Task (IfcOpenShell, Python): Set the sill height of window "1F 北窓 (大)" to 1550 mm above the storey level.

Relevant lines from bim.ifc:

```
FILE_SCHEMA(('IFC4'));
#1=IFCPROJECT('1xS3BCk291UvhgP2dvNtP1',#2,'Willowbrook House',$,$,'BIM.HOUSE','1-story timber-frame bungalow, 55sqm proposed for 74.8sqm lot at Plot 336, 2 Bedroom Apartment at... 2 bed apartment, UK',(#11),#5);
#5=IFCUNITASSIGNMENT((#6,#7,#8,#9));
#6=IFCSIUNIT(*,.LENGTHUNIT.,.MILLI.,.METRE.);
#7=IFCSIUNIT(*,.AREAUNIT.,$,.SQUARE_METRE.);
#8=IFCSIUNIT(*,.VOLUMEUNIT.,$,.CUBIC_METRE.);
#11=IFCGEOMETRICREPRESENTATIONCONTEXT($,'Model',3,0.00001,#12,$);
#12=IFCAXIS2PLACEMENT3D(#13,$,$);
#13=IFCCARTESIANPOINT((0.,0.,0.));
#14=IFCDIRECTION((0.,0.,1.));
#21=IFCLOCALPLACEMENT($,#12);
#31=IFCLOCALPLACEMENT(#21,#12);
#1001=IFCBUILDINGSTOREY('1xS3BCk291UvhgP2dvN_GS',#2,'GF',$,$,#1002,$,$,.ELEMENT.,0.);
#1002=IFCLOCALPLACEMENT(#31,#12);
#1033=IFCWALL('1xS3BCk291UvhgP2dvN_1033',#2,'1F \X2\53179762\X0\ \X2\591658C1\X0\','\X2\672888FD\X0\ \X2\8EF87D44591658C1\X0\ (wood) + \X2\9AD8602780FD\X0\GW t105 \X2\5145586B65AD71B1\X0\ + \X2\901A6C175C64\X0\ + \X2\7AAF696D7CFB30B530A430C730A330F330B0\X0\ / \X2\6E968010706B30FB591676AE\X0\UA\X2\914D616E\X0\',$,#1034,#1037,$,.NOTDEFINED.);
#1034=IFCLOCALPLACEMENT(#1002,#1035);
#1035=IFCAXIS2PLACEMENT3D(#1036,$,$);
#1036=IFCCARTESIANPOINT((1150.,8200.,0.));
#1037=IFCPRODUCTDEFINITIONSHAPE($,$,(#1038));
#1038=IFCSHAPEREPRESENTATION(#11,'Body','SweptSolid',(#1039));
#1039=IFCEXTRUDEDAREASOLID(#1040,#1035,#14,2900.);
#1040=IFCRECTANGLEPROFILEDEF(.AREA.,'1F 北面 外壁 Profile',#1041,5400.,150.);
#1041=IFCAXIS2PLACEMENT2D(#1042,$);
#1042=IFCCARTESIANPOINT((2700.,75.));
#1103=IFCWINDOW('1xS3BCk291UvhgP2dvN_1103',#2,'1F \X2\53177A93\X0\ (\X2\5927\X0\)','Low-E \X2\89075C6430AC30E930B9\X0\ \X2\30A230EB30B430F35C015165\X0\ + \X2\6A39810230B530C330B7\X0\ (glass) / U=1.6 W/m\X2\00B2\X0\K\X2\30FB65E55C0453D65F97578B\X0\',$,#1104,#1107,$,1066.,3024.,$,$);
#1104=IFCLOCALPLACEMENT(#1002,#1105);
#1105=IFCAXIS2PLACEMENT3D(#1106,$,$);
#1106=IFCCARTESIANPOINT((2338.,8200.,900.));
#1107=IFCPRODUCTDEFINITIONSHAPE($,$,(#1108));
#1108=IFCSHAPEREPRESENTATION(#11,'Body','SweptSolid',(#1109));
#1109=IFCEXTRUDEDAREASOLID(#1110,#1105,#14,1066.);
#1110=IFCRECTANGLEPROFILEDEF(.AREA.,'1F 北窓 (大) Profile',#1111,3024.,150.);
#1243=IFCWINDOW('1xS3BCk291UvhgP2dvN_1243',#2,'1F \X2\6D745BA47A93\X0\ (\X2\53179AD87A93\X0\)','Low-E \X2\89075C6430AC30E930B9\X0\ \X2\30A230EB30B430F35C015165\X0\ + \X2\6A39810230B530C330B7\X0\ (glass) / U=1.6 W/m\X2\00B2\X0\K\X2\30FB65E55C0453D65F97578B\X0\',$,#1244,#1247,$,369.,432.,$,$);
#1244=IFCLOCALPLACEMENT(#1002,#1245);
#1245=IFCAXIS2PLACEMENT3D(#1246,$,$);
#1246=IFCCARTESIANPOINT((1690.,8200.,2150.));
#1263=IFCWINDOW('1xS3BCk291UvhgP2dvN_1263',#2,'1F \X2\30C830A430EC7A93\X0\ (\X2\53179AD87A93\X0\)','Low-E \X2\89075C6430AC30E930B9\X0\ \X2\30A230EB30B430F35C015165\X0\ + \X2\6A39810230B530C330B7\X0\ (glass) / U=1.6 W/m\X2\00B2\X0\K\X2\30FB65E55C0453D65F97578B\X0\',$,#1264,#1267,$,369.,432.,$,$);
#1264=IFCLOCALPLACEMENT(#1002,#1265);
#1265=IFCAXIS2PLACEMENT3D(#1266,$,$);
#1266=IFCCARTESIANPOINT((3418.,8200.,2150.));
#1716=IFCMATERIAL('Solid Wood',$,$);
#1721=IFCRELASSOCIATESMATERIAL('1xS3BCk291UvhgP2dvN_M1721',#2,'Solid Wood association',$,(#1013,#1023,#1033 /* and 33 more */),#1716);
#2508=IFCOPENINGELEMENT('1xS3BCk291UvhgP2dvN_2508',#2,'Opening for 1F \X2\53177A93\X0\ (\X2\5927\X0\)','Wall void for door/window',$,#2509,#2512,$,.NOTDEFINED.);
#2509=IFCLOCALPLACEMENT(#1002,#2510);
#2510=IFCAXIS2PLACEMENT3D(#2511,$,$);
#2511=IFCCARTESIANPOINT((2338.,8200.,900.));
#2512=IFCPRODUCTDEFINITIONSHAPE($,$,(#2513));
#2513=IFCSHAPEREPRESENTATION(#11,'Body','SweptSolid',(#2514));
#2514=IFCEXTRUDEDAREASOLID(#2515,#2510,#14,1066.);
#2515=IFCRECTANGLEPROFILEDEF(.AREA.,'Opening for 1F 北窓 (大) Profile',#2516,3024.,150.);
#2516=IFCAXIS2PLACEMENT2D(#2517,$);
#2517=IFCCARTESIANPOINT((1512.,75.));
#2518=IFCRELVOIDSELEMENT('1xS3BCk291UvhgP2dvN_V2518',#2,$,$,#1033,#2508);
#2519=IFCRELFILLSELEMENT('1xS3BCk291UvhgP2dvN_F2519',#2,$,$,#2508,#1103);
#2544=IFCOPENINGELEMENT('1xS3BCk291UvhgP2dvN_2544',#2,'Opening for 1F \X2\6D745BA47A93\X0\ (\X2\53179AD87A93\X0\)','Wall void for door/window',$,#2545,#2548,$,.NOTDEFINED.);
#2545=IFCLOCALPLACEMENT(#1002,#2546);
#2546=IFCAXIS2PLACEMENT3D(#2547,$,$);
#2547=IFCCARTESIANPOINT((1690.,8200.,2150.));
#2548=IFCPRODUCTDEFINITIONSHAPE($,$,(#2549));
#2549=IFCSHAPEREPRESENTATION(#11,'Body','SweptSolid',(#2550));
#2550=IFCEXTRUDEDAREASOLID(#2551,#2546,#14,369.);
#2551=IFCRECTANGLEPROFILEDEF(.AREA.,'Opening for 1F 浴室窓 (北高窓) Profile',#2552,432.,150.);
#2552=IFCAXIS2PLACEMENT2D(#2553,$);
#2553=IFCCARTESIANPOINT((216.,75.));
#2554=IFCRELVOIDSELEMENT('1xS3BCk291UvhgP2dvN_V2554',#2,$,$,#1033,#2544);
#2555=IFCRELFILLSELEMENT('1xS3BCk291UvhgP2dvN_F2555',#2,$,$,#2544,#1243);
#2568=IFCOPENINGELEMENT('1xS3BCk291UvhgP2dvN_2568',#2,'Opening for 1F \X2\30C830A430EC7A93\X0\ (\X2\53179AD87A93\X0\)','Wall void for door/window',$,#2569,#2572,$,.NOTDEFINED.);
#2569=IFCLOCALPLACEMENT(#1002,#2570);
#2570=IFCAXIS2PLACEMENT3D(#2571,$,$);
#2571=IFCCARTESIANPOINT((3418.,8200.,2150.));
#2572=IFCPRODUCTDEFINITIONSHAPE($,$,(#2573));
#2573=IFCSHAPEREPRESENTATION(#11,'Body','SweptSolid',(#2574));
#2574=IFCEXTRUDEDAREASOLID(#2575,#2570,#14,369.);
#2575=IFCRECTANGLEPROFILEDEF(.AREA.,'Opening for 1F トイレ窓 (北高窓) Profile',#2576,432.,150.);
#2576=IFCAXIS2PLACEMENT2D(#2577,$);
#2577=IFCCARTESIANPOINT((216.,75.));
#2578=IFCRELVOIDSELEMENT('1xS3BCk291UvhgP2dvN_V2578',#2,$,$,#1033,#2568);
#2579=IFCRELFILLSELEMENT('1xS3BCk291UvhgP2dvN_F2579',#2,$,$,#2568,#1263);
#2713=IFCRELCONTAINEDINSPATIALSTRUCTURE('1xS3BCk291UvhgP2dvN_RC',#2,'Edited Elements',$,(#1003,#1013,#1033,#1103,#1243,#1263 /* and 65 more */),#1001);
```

```python
import numpy as np
import ifcopenshell
import ifcopenshell.api.geometry
import ifcopenshell.geom
import ifcopenshell.util.element
import ifcopenshell.util.placement
import ifcopenshell.util.shape
import ifcopenshell.util.unit

model = ifcopenshell.open("bim.ifc")
unit_scale = ifcopenshell.util.unit.calculate_unit_scale(model)

window = model.by_id(1103)
opening = window.FillsVoids[0].RelatingOpeningElement
storey = ifcopenshell.util.element.get_container(window, ifc_class="IfcBuildingStorey")
level = ifcopenshell.util.placement.get_local_placement(storey.ObjectPlacement)[2, 3]

# The opening's origin need not be at the sill, so measure its lowest point.
shape = ifcopenshell.geom.create_shape(ifcopenshell.geom.settings(), opening)
bottom = ifcopenshell.util.shape.get_shape_bottom_elevation(shape, shape.geometry) / unit_scale
dz = level + 1550.0 - bottom

shift = np.array([0.0, 0.0, dz])
# The window is not placed relative to its opening, so move both.
for product in (opening, window):
    matrix = ifcopenshell.util.placement.get_local_placement(product.ObjectPlacement)
    matrix[:3, 3] += shift
    ifcopenshell.api.geometry.edit_object_placement(model, product=product, matrix=matrix, is_si=False)

print(f"moved by {dz * unit_scale:+.3f} m")

model.write("bim_v2.ifc")
```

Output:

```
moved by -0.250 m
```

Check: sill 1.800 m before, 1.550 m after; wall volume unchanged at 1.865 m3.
